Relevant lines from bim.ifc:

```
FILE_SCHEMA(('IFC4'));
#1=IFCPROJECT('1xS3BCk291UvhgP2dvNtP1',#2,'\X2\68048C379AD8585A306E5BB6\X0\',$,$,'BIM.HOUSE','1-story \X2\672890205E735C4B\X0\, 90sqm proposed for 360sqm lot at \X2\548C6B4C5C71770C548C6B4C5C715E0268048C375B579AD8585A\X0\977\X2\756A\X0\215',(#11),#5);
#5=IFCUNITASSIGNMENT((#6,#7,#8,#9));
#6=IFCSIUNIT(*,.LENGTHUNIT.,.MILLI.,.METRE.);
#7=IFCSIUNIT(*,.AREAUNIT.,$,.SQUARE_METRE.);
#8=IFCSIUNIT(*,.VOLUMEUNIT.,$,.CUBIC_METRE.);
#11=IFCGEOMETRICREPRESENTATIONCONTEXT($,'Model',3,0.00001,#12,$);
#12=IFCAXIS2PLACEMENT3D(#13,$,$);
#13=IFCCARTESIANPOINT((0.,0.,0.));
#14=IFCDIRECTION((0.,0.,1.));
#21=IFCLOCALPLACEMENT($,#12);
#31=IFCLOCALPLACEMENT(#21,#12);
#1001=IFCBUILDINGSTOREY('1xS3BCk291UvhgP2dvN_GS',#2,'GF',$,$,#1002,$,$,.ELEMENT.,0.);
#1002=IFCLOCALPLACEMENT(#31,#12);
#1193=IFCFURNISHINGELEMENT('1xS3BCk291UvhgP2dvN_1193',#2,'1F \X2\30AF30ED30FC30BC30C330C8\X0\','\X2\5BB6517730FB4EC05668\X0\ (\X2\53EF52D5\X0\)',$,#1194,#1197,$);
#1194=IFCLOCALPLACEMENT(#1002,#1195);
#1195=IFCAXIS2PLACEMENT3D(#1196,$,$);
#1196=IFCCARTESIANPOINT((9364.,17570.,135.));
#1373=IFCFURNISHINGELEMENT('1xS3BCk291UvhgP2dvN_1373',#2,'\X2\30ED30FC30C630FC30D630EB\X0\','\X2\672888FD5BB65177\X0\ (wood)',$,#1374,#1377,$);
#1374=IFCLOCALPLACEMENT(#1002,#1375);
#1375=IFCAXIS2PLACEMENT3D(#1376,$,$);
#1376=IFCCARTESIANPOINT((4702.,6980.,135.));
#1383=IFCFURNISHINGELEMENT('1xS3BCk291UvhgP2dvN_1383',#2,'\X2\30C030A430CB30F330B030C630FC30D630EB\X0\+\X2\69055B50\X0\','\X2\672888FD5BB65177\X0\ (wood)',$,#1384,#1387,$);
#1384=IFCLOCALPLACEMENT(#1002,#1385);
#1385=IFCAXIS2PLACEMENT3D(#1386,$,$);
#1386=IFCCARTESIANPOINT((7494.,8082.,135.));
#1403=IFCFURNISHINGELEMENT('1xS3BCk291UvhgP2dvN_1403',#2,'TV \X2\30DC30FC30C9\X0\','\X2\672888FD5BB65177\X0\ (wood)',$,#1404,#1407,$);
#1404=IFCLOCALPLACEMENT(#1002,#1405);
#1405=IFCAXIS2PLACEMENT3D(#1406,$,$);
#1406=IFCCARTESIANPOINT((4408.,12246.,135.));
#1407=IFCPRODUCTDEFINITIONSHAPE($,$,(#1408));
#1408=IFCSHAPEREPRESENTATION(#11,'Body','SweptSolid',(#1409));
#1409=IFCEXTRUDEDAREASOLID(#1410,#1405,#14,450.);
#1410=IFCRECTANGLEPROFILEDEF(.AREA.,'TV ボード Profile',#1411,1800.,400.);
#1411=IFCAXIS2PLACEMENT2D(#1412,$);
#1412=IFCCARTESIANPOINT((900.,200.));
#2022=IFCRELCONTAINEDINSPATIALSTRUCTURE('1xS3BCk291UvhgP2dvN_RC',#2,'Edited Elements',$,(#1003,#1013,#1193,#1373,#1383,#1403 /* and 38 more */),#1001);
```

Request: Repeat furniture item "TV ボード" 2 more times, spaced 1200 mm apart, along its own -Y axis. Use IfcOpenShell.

```python
import ifcopenshell
import ifcopenshell.api.geometry
import ifcopenshell.api.root
import ifcopenshell.util.element
import ifcopenshell.util.placement

model = ifcopenshell.open("bim.ifc")


def reuse_history(source, copy):
    """copy_class also copies each property set's owner history, people and application; keep the originals."""
    for rel in copy.IsDefinedBy:
        if rel.is_a("IfcRelDefinesByProperties") and (history := rel.RelatingPropertyDefinition.OwnerHistory):
            rel.RelatingPropertyDefinition.OwnerHistory = source.OwnerHistory
            ifcopenshell.util.element.remove_deep2(model, history)


source = model.by_id(1403)
base = ifcopenshell.util.placement.get_local_placement(source.ObjectPlacement)
step = -base[:3, 1] * 1200.0

for i in range(1, 3):
    copy = ifcopenshell.api.root.copy_class(model, product=source)
    copy.Representation = ifcopenshell.util.element.copy_deep(
        model, source.Representation, exclude=["IfcGeometricRepresentationContext", "IfcRepresentationMap"]
    )
    reuse_history(source, copy)
    matrix = base.copy()
    matrix[:3, 3] += i * step
    print("added at", matrix[:3, 3].round(3) + 0.0)
    ifcopenshell.api.geometry.edit_object_placement(model, product=copy, matrix=matrix, is_si=False)

model.write("bim_rev.ifc")
```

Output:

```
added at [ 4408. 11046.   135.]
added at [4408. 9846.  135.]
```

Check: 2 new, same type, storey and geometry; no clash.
